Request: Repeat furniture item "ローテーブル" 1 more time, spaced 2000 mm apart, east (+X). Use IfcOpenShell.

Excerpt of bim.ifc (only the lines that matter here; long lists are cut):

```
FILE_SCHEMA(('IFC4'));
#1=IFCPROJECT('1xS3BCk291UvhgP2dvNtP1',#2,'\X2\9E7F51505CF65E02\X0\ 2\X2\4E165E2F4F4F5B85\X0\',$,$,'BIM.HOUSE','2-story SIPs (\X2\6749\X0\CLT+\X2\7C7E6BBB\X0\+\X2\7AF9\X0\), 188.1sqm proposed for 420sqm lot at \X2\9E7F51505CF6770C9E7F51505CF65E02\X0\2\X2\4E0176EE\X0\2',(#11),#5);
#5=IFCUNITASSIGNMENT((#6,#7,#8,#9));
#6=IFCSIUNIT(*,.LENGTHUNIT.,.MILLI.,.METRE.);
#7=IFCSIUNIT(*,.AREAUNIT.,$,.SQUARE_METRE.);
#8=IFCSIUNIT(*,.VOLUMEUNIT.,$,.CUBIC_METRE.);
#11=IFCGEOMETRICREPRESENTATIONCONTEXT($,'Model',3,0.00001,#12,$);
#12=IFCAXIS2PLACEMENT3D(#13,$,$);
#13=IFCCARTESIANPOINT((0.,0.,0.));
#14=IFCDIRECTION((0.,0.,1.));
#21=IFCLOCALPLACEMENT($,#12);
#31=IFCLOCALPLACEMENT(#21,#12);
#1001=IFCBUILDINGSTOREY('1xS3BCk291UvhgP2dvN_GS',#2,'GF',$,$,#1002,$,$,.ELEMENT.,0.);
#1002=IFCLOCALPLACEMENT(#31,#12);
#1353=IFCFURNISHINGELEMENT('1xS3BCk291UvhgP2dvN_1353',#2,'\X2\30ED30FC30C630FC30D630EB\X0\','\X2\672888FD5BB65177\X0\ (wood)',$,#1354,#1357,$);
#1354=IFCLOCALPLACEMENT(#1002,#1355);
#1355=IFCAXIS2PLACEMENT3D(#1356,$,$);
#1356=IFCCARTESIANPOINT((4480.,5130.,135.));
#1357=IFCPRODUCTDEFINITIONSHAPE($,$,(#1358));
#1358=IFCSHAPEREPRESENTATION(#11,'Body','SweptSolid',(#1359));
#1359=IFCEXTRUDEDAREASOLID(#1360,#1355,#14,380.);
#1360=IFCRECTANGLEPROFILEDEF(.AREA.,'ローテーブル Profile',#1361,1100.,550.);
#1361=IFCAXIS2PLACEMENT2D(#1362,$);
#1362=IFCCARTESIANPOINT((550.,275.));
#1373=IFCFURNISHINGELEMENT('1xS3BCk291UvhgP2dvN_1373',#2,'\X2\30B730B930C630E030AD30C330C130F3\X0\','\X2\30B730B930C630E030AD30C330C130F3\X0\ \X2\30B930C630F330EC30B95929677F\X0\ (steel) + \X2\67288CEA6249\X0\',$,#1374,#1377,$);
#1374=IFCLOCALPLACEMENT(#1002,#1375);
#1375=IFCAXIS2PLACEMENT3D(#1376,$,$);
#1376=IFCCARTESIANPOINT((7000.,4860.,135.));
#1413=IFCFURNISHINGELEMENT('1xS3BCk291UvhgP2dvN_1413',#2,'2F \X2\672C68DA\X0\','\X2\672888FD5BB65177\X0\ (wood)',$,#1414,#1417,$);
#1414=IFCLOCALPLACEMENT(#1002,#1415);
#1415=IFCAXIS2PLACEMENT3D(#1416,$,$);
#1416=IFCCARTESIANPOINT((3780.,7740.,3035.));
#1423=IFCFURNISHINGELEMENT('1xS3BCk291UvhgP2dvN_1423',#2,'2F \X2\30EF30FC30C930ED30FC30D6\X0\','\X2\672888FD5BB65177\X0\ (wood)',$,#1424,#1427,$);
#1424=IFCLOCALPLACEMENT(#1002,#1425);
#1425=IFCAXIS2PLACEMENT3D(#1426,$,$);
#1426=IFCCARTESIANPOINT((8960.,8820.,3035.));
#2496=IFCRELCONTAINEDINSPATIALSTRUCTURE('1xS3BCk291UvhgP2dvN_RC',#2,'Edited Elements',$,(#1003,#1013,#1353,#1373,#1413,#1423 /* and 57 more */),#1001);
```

```python
import numpy as np
import ifcopenshell
import ifcopenshell.api.geometry
import ifcopenshell.api.root
import ifcopenshell.util.element
import ifcopenshell.util.placement
import ifcopenshell.util.unit

model = ifcopenshell.open("bim.ifc")
unit_scale = ifcopenshell.util.unit.calculate_unit_scale(model)


def reuse_history(source, copy):
    """copy_class also copies each property set's owner history, people and application; keep the originals."""
    for rel in copy.IsDefinedBy:
        if rel.is_a("IfcRelDefinesByProperties") and (history := rel.RelatingPropertyDefinition.OwnerHistory):
            rel.RelatingPropertyDefinition.OwnerHistory = source.OwnerHistory
            ifcopenshell.util.element.remove_deep2(model, history)


source = model.by_guid("1xS3BCk291UvhgP2dvN_1353")
base = ifcopenshell.util.placement.get_local_placement(source.ObjectPlacement)
step = np.array([1.0, 0.0, 0.0]) * 2 / unit_scale

for i in range(1, 2):
    copy = ifcopenshell.api.root.copy_class(model, product=source)
    copy.Representation = ifcopenshell.util.element.copy_deep(
        model, source.Representation, exclude=["IfcGeometricRepresentationContext", "IfcRepresentationMap"]
    )
    reuse_history(source, copy)
    matrix = base.copy()
    matrix[:3, 3] += i * step
    print("added at", matrix[:3, 3].round(3) + 0.0)
    ifcopenshell.api.geometry.edit_object_placement(model, product=copy, matrix=matrix, is_si=False)

model.write("bim_edited.ifc")
```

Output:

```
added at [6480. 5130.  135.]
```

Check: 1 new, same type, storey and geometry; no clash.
